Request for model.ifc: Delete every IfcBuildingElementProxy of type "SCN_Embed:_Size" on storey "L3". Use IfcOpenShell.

First a look at what the model holds.

```python
import ifcopenshell
import ifcopenshell.util.element

model = ifcopenshell.open("model.ifc")
print(model.schema)
storey = next(s for s in model.by_type("IfcBuildingStorey") if s.Name == "L3")
proxies = [e for e in ifcopenshell.util.element.get_decomposition(storey) if e.is_a("IfcBuildingElementProxy")]
seen = {}
for e in proxies:
    element_type = ifcopenshell.util.element.get_type(e)
    name = element_type.Name if element_type not in (None, e) else None
    seen[name] = seen.get(name, 0) + 1
for name, count in sorted(seen.items(), key=str):
    print(count, "x", name)
```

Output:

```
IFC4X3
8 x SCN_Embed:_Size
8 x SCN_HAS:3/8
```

```python
import ifcopenshell
import ifcopenshell.api.root
import ifcopenshell.util.element

model = ifcopenshell.open("model.ifc")

storey = next(s for s in model.by_type("IfcBuildingStorey") if s.Name == "L3")
proxies = [e for e in ifcopenshell.util.element.get_decomposition(storey) if e.is_a("IfcBuildingElementProxy")]
targets = [e for e in proxies if (t := ifcopenshell.util.element.get_type(e)) not in (None, e) and t.Name == "SCN_Embed:_Size"]

for e in targets:
    ifcopenshell.api.root.remove_product(model, product=e)
print(len(targets), "removed")

model.write("model-out.ifc")
```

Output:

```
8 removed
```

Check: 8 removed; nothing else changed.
